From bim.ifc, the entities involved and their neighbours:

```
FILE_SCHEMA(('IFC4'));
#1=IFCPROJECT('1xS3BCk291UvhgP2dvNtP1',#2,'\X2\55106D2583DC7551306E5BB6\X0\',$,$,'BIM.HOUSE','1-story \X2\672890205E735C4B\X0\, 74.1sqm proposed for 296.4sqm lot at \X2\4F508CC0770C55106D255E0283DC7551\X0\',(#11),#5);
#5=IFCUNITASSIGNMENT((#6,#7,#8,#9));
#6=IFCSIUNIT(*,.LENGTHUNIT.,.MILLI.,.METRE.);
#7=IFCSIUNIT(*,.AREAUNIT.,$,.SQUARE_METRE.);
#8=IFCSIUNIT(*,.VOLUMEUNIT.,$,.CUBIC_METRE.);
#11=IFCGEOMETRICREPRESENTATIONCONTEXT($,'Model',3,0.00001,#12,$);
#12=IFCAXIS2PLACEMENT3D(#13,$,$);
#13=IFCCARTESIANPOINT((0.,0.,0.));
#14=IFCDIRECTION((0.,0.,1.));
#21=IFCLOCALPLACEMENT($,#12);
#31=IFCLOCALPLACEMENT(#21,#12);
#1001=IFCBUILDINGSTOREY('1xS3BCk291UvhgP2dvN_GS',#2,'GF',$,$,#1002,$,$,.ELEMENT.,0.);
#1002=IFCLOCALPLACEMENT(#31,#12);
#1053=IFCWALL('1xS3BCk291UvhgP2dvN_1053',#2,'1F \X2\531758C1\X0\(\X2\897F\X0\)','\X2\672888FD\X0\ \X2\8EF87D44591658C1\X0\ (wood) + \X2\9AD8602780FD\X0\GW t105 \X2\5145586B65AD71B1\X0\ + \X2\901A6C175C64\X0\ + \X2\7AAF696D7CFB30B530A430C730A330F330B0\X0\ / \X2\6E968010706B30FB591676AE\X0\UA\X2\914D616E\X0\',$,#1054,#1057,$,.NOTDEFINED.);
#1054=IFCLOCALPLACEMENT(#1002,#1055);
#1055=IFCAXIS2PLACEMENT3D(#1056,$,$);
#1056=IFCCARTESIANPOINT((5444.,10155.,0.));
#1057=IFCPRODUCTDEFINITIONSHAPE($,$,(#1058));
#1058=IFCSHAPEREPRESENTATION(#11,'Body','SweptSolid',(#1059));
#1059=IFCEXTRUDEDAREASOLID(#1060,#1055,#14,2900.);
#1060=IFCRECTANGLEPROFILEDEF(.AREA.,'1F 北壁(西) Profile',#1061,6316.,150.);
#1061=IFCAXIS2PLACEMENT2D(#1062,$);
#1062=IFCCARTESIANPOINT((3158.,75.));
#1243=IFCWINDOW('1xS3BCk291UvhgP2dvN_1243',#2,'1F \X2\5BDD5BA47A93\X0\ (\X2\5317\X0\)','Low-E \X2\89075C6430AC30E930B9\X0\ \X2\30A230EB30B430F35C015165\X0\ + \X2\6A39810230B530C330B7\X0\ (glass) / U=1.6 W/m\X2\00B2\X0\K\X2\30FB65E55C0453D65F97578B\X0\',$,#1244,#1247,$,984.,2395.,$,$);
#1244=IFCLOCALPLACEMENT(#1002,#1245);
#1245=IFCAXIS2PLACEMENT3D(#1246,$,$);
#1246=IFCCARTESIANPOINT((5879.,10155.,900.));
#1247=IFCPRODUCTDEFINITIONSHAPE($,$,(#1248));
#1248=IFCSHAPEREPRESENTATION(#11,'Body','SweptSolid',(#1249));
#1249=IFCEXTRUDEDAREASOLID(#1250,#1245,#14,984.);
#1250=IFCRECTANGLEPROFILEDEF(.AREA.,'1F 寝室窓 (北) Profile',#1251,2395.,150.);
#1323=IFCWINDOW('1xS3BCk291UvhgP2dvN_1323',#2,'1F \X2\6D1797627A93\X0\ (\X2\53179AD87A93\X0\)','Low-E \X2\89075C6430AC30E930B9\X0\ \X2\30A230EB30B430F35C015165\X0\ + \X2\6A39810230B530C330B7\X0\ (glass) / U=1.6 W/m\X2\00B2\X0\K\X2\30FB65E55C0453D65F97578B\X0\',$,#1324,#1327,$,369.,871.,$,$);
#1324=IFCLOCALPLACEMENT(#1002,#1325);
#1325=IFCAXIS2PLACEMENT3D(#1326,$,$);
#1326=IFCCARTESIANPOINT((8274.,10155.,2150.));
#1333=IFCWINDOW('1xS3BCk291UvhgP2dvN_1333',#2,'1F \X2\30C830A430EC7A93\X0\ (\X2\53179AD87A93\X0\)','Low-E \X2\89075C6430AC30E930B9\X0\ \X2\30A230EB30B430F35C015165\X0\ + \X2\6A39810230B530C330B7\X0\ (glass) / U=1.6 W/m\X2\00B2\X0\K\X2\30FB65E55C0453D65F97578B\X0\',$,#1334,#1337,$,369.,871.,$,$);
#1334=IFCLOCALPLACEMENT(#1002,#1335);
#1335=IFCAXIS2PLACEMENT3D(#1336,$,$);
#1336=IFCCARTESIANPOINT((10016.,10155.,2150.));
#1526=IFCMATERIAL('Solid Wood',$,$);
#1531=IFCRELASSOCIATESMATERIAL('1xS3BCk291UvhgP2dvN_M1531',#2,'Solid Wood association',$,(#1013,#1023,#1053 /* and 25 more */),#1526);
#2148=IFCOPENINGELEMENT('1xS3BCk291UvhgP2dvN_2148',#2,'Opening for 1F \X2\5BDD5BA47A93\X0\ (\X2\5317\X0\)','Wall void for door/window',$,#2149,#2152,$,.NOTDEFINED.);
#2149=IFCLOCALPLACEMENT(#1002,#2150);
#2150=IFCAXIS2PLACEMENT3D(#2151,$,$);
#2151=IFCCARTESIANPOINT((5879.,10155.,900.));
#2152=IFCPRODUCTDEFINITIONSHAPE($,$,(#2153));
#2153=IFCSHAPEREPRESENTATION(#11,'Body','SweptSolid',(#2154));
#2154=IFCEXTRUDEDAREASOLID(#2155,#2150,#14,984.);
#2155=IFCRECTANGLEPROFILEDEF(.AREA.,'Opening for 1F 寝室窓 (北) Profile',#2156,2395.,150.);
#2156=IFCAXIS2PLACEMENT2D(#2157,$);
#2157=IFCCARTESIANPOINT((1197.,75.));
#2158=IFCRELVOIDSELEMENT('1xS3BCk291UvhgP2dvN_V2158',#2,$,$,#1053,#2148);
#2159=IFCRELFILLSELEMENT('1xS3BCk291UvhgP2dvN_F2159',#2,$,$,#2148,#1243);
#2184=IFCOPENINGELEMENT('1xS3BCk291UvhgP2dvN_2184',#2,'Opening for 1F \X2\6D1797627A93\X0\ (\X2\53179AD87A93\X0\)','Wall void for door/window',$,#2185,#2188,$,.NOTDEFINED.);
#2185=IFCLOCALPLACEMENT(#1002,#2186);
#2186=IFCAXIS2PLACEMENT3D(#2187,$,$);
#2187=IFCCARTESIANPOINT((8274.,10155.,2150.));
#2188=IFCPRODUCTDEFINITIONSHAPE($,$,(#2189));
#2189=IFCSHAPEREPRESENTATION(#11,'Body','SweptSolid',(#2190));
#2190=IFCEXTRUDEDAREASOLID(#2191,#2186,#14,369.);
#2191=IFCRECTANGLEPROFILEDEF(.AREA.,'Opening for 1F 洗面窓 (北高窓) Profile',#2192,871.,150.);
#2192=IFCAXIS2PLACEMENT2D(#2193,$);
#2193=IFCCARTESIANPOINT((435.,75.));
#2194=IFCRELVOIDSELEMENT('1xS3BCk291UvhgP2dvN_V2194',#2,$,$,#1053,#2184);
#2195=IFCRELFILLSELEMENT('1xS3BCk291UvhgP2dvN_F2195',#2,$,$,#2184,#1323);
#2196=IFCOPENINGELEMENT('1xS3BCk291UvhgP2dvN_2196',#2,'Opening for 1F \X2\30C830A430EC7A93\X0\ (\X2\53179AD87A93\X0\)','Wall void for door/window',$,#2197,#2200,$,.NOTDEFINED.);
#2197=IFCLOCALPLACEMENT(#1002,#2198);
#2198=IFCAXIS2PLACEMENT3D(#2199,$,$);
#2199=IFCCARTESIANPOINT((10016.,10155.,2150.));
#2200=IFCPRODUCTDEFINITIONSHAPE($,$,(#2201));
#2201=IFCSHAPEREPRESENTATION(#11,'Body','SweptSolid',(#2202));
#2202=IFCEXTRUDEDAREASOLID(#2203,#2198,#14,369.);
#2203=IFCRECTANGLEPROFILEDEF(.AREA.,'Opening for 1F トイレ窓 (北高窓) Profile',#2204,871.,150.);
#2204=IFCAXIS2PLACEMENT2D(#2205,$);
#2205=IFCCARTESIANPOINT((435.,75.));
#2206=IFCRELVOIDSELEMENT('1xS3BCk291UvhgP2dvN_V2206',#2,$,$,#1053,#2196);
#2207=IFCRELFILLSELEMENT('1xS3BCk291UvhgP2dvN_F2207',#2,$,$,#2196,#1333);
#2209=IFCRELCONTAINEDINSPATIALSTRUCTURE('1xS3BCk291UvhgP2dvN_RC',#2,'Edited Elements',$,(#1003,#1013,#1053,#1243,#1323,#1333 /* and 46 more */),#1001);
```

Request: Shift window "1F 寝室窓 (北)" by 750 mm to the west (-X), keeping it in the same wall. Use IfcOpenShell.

```python
import ifcopenshell
import ifcopenshell.api.geometry
import ifcopenshell.util.placement

model = ifcopenshell.open("bim.ifc")

window = model.by_id(1243)
opening = window.FillsVoids[0].RelatingOpeningElement
wall = opening.VoidsElements[0].RelatingBuildingElement

wall_matrix = ifcopenshell.util.placement.get_local_placement(wall.ObjectPlacement)
shift = wall_matrix[:3, 0] * -750.0
before = ifcopenshell.util.placement.get_local_placement(window.ObjectPlacement)[:3, 3].copy()

# The window is not placed relative to its opening, so move both.
for product in (opening, window):
    matrix = ifcopenshell.util.placement.get_local_placement(product.ObjectPlacement)
    matrix[:3, 3] += shift
    ifcopenshell.api.geometry.edit_object_placement(model, product=product, matrix=matrix, is_si=False)

after = ifcopenshell.util.placement.get_local_placement(window.ObjectPlacement)[:3, 3]
print("window moved by", (after - before).round(3) + 0.0)

model.write("bim_v2.ifc")
```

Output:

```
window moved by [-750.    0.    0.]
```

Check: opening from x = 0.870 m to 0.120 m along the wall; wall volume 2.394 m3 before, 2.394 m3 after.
